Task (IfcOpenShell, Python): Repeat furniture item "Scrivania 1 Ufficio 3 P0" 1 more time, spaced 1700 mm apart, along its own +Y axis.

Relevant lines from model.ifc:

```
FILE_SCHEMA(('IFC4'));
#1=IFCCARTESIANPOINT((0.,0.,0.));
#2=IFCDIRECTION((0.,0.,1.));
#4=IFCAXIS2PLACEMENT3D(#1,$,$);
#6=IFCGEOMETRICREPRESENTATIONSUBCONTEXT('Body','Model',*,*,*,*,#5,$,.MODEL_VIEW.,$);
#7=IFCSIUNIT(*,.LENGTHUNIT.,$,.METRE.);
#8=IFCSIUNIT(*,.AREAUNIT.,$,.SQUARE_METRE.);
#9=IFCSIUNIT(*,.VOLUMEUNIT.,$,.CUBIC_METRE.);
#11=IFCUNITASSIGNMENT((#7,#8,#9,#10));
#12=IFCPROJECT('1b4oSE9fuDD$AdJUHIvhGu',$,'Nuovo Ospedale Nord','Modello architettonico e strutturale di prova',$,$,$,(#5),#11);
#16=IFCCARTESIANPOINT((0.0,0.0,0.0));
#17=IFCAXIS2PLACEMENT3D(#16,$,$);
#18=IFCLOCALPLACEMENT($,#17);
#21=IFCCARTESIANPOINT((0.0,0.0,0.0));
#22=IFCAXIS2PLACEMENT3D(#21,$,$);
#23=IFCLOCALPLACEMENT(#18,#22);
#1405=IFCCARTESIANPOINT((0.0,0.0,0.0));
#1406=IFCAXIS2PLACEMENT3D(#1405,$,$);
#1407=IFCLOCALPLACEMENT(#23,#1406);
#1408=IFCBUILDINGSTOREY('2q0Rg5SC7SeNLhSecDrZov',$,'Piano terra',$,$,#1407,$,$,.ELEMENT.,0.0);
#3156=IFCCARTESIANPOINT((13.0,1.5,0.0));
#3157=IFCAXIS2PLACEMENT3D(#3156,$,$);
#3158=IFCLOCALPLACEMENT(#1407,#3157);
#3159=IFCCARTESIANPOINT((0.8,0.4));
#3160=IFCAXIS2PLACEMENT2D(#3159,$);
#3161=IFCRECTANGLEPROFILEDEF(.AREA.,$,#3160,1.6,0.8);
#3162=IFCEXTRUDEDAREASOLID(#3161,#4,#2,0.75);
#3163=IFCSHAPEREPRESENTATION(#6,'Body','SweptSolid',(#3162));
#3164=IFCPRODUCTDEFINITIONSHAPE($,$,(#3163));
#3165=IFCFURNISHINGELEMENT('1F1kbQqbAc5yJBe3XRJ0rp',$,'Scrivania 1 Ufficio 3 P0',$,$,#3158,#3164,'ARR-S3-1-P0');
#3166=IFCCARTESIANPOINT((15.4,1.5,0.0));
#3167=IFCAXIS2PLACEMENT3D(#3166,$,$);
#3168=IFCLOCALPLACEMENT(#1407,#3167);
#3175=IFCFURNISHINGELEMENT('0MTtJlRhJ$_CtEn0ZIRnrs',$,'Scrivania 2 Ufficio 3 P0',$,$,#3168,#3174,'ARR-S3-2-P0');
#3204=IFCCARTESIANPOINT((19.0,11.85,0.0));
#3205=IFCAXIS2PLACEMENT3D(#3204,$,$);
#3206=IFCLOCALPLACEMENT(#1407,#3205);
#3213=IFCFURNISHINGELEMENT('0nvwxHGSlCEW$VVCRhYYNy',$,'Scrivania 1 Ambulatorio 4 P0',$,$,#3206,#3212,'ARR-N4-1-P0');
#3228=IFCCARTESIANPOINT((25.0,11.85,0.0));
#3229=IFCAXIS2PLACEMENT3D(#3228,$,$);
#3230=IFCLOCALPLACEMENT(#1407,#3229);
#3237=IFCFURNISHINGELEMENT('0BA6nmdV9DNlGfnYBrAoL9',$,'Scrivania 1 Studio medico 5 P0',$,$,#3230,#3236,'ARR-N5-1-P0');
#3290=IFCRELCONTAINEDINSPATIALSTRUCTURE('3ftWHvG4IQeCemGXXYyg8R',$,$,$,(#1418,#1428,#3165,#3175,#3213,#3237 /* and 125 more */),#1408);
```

```python
import ifcopenshell
import ifcopenshell.api.geometry
import ifcopenshell.api.root
import ifcopenshell.util.element
import ifcopenshell.util.placement
import ifcopenshell.util.unit

model = ifcopenshell.open("model.ifc")
unit_scale = ifcopenshell.util.unit.calculate_unit_scale(model)

source = model.by_guid("1F1kbQqbAc5yJBe3XRJ0rp")
base = ifcopenshell.util.placement.get_local_placement(source.ObjectPlacement)
step = base[:3, 1] * 1.7 / unit_scale

for i in range(1, 2):
    copy = ifcopenshell.api.root.copy_class(model, product=source)
    copy.Representation = ifcopenshell.util.element.copy_deep(
        model, source.Representation, exclude=["IfcGeometricRepresentationContext", "IfcRepresentationMap"]
    )
    copy.Tag = None
    matrix = base.copy()
    matrix[:3, 3] += i * step
    print("added at", matrix[:3, 3].round(3) + 0.0)
    ifcopenshell.api.geometry.edit_object_placement(model, product=copy, matrix=matrix, is_si=False)

model.write("model_updated.ifc")
```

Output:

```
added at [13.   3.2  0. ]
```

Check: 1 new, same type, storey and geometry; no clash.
